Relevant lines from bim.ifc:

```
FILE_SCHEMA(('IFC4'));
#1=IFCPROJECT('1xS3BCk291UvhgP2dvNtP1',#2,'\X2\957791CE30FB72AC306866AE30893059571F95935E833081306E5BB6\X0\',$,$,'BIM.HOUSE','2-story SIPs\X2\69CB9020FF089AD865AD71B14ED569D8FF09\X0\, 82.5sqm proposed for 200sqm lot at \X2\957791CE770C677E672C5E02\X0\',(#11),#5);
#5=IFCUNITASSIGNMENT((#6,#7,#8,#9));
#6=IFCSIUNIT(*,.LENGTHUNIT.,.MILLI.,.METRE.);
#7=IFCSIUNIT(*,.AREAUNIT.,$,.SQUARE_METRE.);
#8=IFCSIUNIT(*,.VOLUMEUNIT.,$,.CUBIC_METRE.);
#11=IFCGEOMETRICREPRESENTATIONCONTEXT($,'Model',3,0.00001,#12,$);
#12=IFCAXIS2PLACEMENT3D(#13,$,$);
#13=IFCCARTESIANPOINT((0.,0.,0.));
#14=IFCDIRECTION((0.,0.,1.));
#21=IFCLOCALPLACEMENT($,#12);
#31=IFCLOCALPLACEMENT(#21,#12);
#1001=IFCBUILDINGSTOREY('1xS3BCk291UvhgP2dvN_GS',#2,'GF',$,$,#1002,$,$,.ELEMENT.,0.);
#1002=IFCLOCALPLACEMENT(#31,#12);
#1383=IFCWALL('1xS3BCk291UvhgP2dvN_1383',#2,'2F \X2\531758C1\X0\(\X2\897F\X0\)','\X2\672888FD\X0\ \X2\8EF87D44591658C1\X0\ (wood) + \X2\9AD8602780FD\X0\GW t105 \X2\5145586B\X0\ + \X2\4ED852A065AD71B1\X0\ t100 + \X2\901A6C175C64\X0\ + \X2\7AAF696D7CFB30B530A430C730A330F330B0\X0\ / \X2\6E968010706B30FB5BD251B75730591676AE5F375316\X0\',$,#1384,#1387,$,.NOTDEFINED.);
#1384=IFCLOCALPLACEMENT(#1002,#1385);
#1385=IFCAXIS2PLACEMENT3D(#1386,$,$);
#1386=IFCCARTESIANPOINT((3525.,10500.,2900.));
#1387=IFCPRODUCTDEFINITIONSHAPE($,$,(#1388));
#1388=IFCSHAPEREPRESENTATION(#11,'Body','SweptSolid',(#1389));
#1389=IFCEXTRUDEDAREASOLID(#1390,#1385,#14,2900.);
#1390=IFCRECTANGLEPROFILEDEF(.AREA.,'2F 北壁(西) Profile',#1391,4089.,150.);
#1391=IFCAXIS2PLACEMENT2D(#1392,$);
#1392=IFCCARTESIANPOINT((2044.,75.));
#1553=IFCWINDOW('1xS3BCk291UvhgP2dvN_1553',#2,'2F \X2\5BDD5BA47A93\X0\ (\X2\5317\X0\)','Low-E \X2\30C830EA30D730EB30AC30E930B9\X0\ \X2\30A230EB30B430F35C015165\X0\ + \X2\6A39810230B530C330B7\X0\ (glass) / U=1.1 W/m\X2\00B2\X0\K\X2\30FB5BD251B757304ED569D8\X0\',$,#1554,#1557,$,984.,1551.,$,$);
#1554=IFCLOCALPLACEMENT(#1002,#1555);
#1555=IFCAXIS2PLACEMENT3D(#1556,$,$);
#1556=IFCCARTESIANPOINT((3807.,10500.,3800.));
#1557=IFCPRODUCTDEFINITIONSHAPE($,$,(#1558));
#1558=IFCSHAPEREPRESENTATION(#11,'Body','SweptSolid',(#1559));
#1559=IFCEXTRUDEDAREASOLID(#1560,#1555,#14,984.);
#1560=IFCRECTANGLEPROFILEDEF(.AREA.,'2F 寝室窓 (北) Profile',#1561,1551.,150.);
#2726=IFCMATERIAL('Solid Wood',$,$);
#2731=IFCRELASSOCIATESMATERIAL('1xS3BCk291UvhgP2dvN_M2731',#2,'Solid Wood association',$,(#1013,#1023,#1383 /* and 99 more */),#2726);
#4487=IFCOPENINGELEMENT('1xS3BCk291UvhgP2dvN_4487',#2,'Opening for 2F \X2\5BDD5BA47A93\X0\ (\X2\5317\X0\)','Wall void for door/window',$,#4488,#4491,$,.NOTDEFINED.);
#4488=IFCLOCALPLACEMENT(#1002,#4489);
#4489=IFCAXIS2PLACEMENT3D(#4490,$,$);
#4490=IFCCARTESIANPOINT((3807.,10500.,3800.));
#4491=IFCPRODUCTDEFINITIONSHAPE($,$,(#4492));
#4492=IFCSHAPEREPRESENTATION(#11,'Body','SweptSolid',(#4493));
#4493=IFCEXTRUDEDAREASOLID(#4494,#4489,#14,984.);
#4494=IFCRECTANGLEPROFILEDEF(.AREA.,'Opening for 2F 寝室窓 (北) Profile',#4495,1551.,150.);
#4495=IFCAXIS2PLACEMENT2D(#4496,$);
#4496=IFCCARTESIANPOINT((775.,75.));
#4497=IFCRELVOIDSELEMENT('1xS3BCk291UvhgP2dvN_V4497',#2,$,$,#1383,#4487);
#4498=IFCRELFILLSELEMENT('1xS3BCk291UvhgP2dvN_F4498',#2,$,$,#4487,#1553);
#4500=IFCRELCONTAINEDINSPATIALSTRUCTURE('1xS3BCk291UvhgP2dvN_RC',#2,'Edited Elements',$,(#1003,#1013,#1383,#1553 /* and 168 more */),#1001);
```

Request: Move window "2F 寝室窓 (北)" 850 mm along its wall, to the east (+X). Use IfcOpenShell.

```python
import ifcopenshell
import ifcopenshell.api.geometry
import ifcopenshell.util.placement
import ifcopenshell.util.unit

model = ifcopenshell.open("bim.ifc")
unit_scale = ifcopenshell.util.unit.calculate_unit_scale(model)

window = model.by_id(1553)
opening = window.FillsVoids[0].RelatingOpeningElement
wall = opening.VoidsElements[0].RelatingBuildingElement

wall_matrix = ifcopenshell.util.placement.get_local_placement(wall.ObjectPlacement)
shift = wall_matrix[:3, 0] * 0.85 / unit_scale
before = ifcopenshell.util.placement.get_local_placement(window.ObjectPlacement)[:3, 3].copy()

# The window is not placed relative to its opening, so move both.
for product in (opening, window):
    matrix = ifcopenshell.util.placement.get_local_placement(product.ObjectPlacement)
    matrix[:3, 3] += shift
    ifcopenshell.api.geometry.edit_object_placement(model, product=product, matrix=matrix, is_si=False)

after = ifcopenshell.util.placement.get_local_placement(window.ObjectPlacement)[:3, 3]
print("window moved by", (after - before).round(3) + 0.0)

model.write("bim_updated.ifc")
```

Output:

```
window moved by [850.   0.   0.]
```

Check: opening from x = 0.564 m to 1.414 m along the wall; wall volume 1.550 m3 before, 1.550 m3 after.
